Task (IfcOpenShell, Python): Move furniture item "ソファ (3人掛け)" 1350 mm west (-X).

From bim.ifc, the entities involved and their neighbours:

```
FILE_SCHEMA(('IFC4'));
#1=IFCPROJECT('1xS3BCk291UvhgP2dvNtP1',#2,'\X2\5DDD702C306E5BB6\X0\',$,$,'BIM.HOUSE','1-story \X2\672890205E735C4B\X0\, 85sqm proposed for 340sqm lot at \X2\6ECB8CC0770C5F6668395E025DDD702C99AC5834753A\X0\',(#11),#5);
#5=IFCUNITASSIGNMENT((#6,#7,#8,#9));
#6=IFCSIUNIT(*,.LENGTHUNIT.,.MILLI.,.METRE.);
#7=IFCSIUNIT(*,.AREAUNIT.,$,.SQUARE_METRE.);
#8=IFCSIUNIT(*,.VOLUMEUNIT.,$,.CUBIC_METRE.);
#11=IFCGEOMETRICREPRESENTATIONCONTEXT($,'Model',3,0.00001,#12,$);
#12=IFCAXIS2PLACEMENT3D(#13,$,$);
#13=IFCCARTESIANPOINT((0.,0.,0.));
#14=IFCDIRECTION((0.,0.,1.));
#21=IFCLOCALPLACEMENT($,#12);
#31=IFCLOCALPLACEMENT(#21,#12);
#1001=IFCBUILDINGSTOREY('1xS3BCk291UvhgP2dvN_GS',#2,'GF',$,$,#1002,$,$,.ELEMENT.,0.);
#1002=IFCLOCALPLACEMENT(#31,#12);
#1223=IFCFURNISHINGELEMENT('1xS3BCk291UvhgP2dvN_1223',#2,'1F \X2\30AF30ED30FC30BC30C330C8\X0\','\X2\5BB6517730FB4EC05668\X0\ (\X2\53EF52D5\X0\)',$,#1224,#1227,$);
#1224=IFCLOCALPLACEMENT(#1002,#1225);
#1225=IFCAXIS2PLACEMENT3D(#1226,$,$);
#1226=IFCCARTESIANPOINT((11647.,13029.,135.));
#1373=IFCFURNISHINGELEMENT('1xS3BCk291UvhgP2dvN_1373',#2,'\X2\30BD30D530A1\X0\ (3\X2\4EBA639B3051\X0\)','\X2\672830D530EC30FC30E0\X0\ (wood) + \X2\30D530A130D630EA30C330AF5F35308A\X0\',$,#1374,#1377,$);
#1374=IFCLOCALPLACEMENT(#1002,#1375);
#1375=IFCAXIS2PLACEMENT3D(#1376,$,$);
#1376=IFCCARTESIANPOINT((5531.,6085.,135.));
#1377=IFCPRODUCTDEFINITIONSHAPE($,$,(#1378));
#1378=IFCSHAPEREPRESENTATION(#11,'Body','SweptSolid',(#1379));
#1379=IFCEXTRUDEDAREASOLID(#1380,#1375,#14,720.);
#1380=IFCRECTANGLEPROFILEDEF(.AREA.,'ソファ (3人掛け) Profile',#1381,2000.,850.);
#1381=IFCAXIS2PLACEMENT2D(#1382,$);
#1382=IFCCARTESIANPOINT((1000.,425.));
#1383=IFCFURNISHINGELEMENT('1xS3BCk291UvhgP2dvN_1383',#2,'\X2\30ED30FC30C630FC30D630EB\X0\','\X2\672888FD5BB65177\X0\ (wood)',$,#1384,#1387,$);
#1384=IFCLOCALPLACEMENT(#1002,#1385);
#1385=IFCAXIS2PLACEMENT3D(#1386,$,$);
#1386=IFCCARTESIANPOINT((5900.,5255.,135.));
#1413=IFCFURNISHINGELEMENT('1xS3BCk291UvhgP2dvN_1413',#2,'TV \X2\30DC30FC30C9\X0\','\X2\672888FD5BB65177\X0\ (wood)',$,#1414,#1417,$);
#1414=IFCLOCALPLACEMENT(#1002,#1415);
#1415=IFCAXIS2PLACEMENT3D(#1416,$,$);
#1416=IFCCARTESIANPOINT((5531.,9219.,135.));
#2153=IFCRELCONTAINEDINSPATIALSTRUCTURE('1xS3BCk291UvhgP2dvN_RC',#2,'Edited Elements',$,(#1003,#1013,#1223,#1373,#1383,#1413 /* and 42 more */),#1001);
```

```python
import ifcopenshell
import ifcopenshell.api.geometry
import ifcopenshell.util.placement

model = ifcopenshell.open("bim.ifc")

item = model.by_id(1373)
matrix = ifcopenshell.util.placement.get_local_placement(item.ObjectPlacement)
matrix[0, 3] -= 1350.0
ifcopenshell.api.geometry.edit_object_placement(model, product=item, matrix=matrix, is_si=False)

print(ifcopenshell.util.placement.get_local_placement(item.ObjectPlacement).round(3) + 0.0)

model.write("bim-out.ifc")
```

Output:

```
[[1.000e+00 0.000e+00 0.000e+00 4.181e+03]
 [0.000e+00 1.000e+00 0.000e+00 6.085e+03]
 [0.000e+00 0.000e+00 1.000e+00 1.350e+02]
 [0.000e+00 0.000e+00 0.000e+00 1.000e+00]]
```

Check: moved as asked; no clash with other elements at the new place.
